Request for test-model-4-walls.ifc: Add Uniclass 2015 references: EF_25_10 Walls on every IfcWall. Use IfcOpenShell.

First a look at what the model holds.

```python
import ifcopenshell

model = ifcopenshell.open("test-model-4-walls.ifc")
print(model.schema)
print("classifications:", [c.Name for c in model.by_type("IfcClassification")])
for ifc_class in ("IfcDoor", "IfcRoof", "IfcStair", "IfcWall", "IfcWindow"):
    print(ifc_class, len(model.by_type(ifc_class)))
```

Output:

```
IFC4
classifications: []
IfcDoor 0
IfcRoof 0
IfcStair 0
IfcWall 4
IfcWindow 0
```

```python
import ifcopenshell
import ifcopenshell.api.classification

model = ifcopenshell.open("test-model-4-walls.ifc")

system = ifcopenshell.api.classification.add_classification(model, classification="Uniclass 2015")

codes = {
    "IfcWall": ("EF_25_10", "Walls"),
}
for ifc_class, (code, name) in codes.items():
    products = model.by_type(ifc_class)
    ifcopenshell.api.classification.add_reference(
        model, products=products, classification=system, identification=code, name=name
    )
    print(code, len(products))

model.write("test-model-4-walls-out.ifc")
```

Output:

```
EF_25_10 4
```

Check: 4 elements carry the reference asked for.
